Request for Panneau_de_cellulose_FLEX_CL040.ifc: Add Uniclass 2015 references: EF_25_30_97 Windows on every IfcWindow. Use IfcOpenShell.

First a look at what the model holds.

```python
import ifcopenshell

model = ifcopenshell.open("Panneau_de_cellulose_FLEX_CL040.ifc")
print(model.schema)
print("classifications:", [c.Name for c in model.by_type("IfcClassification")])
for ifc_class in ("IfcDoor", "IfcRoof", "IfcStair", "IfcWall", "IfcWindow"):
    print(ifc_class, len(model.by_type(ifc_class)))
```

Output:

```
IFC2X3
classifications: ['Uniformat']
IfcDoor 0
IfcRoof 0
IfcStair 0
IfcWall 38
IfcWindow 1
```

```python
import ifcopenshell
import ifcopenshell.api.classification

model = ifcopenshell.open("Panneau_de_cellulose_FLEX_CL040.ifc")

# IFC2X3 requires Source and Edition and has no link from the project to the system.
system = model.create_entity("IfcClassification", Source="NBS", Edition="2015", Name="Uniclass 2015")

codes = {
    "IfcWindow": ("EF_25_30_97", "Windows"),
}
for ifc_class, (code, name) in codes.items():
    products = model.by_type(ifc_class)
    ifcopenshell.api.classification.add_reference(
        model, products=products, classification=system, identification=code, name=name
    )
    print(code, len(products))

model.write("Panneau_de_cellulose_FLEX_CL040_edited.ifc")
```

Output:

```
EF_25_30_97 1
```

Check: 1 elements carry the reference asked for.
